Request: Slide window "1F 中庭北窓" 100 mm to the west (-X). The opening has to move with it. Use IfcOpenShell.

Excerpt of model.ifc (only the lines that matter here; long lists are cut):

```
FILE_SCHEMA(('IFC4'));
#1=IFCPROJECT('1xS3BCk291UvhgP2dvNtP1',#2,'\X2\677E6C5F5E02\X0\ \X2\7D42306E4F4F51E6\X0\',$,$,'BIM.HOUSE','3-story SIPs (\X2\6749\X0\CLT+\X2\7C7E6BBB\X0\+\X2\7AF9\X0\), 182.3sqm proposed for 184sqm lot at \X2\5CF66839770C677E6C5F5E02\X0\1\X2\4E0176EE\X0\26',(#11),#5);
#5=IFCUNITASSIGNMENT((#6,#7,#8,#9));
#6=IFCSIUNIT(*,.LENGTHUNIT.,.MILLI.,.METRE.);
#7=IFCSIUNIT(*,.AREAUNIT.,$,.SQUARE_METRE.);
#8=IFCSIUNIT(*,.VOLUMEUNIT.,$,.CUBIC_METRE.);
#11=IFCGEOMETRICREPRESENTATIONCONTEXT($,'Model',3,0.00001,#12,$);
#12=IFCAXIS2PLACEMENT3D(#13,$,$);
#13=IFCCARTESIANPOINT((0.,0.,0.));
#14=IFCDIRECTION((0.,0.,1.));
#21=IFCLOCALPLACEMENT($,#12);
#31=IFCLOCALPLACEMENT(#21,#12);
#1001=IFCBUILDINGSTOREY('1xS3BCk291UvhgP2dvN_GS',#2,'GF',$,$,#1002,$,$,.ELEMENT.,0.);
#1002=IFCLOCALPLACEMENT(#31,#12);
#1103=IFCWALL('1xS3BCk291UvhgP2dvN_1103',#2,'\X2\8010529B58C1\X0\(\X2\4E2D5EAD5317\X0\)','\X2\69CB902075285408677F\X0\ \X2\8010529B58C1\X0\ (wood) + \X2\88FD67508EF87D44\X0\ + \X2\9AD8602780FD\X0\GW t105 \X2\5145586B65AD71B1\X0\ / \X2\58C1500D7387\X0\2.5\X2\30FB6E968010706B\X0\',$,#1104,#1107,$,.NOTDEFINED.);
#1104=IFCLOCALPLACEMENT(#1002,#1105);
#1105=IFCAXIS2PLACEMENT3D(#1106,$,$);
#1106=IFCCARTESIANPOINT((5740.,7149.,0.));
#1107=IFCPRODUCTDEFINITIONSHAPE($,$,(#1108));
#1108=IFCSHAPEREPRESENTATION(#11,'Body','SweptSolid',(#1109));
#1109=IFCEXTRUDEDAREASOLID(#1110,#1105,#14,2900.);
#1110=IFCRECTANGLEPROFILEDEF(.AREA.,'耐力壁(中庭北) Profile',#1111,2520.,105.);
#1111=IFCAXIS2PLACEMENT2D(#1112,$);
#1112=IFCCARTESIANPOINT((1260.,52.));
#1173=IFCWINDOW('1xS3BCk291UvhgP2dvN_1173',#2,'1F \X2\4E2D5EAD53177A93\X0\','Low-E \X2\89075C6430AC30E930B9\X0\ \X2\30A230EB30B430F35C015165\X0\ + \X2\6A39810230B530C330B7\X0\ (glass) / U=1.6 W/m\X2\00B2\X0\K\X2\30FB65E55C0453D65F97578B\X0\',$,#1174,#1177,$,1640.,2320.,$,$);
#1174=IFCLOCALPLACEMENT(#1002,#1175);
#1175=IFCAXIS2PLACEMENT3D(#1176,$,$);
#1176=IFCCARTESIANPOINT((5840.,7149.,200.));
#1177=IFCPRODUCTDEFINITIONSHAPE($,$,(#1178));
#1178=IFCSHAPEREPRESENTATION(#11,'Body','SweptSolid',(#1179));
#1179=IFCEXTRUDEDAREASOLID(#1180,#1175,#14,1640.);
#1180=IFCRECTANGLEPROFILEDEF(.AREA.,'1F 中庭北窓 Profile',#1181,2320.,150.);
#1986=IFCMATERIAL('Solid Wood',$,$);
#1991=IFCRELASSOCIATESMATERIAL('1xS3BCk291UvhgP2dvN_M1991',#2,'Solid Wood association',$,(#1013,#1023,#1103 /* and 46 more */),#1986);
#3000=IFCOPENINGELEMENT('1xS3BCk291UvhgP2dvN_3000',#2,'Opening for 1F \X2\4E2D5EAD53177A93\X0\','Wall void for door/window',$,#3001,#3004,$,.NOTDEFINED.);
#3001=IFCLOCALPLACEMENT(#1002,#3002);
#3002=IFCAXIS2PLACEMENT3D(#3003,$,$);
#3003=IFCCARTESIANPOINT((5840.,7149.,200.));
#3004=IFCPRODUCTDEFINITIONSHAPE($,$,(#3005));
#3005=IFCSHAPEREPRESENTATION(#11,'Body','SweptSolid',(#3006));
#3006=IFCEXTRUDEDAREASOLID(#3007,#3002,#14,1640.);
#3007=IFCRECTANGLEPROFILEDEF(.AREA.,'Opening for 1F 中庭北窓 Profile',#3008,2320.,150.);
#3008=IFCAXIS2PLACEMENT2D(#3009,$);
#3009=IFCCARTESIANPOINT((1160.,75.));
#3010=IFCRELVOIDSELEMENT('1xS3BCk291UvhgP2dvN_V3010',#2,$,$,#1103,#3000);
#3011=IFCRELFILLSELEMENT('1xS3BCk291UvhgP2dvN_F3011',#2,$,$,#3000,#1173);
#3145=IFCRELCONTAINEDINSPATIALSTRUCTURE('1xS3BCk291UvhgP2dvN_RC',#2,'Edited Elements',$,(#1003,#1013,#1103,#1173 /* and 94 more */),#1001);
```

```python
import ifcopenshell
import ifcopenshell.api.geometry
import ifcopenshell.util.placement
import ifcopenshell.util.unit

model = ifcopenshell.open("model.ifc")
unit_scale = ifcopenshell.util.unit.calculate_unit_scale(model)

window = model.by_id(1173)
opening = window.FillsVoids[0].RelatingOpeningElement
wall = opening.VoidsElements[0].RelatingBuildingElement

wall_matrix = ifcopenshell.util.placement.get_local_placement(wall.ObjectPlacement)
shift = wall_matrix[:3, 0] * -0.1 / unit_scale
before = ifcopenshell.util.placement.get_local_placement(window.ObjectPlacement)[:3, 3].copy()

# The window is not placed relative to its opening, so move both.
for product in (opening, window):
    matrix = ifcopenshell.util.placement.get_local_placement(product.ObjectPlacement)
    matrix[:3, 3] += shift
    ifcopenshell.api.geometry.edit_object_placement(model, product=product, matrix=matrix, is_si=False)

after = ifcopenshell.util.placement.get_local_placement(window.ObjectPlacement)[:3, 3]
print("window moved by", (after - before).round(3) + 0.0)

model.write("model_edited.ifc")
```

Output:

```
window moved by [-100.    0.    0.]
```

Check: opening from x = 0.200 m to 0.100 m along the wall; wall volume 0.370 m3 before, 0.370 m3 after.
